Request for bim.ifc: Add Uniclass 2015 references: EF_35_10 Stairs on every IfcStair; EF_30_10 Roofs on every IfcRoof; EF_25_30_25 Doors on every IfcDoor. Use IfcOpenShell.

First a look at what the model holds.

```python
import ifcopenshell

model = ifcopenshell.open("bim.ifc")
print(model.schema)
print("classifications:", [c.Name for c in model.by_type("IfcClassification")])
for ifc_class in ("IfcDoor", "IfcRoof", "IfcStair", "IfcWall", "IfcWindow"):
    print(ifc_class, len(model.by_type(ifc_class)))
```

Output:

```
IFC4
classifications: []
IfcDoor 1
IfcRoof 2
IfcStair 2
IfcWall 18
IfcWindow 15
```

```python
import ifcopenshell
import ifcopenshell.api.classification

model = ifcopenshell.open("bim.ifc")

system = ifcopenshell.api.classification.add_classification(model, classification="Uniclass 2015")

codes = {
    "IfcStair": ("EF_35_10", "Stairs"),
    "IfcRoof": ("EF_30_10", "Roofs"),
    "IfcDoor": ("EF_25_30_25", "Doors"),
}
for ifc_class, (code, name) in codes.items():
    products = model.by_type(ifc_class)
    ifcopenshell.api.classification.add_reference(
        model, products=products, classification=system, identification=code, name=name
    )
    print(code, len(products))

model.write("bim-out.ifc")
```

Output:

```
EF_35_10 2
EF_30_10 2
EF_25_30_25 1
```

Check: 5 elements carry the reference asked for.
